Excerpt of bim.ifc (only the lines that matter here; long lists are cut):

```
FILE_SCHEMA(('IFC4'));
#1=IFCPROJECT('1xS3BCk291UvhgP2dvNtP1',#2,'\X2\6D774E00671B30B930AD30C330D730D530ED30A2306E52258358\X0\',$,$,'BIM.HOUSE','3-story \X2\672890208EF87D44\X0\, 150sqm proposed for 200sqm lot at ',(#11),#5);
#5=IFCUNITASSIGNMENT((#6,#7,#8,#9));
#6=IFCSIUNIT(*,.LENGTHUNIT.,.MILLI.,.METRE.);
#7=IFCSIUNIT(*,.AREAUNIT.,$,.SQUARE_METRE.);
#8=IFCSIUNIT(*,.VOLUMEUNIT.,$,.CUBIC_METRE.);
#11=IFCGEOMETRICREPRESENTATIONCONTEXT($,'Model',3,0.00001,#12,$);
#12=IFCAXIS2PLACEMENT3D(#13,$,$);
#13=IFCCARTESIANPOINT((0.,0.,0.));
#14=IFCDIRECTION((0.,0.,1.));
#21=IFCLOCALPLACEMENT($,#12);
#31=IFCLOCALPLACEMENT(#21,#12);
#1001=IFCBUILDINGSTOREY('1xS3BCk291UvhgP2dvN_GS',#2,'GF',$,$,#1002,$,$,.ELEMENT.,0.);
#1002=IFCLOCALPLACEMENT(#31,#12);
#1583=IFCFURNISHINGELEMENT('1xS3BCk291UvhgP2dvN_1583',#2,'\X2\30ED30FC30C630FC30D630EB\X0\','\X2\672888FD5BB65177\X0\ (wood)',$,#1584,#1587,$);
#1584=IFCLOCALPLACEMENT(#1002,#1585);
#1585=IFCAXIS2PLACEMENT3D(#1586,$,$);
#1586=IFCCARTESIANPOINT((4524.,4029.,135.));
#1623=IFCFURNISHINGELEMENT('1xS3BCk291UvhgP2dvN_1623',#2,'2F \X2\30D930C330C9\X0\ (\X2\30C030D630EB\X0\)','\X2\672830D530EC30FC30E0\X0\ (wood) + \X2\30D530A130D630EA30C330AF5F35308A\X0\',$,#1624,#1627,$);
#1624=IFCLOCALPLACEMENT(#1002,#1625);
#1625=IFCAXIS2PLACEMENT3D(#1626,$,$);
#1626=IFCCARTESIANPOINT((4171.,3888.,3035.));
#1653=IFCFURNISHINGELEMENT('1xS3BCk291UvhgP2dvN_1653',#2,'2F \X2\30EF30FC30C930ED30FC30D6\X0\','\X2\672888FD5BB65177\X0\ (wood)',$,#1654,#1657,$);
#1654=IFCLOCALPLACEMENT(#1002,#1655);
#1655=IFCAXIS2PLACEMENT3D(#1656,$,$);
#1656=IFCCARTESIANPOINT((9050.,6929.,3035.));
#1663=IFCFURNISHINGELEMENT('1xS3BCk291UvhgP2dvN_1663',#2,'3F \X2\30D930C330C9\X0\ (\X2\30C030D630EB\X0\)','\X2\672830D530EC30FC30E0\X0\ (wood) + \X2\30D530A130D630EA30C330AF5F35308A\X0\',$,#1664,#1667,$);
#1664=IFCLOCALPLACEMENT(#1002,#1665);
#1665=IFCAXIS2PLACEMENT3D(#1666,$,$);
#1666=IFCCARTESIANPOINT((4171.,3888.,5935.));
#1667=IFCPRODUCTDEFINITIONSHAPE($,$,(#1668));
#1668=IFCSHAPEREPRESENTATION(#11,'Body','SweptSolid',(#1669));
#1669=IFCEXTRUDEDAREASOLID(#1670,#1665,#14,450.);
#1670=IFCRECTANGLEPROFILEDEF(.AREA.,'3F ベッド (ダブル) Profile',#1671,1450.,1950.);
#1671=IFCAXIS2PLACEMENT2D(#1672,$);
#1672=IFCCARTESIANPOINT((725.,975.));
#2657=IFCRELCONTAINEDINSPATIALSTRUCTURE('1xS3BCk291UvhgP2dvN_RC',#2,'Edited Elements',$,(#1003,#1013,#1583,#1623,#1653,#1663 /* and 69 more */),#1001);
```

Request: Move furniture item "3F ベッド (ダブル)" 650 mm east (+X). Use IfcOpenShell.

```python
import ifcopenshell
import ifcopenshell.api.geometry
import ifcopenshell.util.placement
import ifcopenshell.util.unit

model = ifcopenshell.open("bim.ifc")
unit_scale = ifcopenshell.util.unit.calculate_unit_scale(model)

item = model.by_guid("1xS3BCk291UvhgP2dvN_1663")
matrix = ifcopenshell.util.placement.get_local_placement(item.ObjectPlacement)
matrix[0, 3] += 0.65 / unit_scale
ifcopenshell.api.geometry.edit_object_placement(model, product=item, matrix=matrix, is_si=False)

print(ifcopenshell.util.placement.get_local_placement(item.ObjectPlacement).round(3) + 0.0)

model.write("bim_v2.ifc")
```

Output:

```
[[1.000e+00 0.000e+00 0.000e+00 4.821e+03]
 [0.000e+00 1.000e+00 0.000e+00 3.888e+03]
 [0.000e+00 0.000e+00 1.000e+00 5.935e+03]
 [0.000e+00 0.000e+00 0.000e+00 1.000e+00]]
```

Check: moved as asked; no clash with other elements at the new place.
